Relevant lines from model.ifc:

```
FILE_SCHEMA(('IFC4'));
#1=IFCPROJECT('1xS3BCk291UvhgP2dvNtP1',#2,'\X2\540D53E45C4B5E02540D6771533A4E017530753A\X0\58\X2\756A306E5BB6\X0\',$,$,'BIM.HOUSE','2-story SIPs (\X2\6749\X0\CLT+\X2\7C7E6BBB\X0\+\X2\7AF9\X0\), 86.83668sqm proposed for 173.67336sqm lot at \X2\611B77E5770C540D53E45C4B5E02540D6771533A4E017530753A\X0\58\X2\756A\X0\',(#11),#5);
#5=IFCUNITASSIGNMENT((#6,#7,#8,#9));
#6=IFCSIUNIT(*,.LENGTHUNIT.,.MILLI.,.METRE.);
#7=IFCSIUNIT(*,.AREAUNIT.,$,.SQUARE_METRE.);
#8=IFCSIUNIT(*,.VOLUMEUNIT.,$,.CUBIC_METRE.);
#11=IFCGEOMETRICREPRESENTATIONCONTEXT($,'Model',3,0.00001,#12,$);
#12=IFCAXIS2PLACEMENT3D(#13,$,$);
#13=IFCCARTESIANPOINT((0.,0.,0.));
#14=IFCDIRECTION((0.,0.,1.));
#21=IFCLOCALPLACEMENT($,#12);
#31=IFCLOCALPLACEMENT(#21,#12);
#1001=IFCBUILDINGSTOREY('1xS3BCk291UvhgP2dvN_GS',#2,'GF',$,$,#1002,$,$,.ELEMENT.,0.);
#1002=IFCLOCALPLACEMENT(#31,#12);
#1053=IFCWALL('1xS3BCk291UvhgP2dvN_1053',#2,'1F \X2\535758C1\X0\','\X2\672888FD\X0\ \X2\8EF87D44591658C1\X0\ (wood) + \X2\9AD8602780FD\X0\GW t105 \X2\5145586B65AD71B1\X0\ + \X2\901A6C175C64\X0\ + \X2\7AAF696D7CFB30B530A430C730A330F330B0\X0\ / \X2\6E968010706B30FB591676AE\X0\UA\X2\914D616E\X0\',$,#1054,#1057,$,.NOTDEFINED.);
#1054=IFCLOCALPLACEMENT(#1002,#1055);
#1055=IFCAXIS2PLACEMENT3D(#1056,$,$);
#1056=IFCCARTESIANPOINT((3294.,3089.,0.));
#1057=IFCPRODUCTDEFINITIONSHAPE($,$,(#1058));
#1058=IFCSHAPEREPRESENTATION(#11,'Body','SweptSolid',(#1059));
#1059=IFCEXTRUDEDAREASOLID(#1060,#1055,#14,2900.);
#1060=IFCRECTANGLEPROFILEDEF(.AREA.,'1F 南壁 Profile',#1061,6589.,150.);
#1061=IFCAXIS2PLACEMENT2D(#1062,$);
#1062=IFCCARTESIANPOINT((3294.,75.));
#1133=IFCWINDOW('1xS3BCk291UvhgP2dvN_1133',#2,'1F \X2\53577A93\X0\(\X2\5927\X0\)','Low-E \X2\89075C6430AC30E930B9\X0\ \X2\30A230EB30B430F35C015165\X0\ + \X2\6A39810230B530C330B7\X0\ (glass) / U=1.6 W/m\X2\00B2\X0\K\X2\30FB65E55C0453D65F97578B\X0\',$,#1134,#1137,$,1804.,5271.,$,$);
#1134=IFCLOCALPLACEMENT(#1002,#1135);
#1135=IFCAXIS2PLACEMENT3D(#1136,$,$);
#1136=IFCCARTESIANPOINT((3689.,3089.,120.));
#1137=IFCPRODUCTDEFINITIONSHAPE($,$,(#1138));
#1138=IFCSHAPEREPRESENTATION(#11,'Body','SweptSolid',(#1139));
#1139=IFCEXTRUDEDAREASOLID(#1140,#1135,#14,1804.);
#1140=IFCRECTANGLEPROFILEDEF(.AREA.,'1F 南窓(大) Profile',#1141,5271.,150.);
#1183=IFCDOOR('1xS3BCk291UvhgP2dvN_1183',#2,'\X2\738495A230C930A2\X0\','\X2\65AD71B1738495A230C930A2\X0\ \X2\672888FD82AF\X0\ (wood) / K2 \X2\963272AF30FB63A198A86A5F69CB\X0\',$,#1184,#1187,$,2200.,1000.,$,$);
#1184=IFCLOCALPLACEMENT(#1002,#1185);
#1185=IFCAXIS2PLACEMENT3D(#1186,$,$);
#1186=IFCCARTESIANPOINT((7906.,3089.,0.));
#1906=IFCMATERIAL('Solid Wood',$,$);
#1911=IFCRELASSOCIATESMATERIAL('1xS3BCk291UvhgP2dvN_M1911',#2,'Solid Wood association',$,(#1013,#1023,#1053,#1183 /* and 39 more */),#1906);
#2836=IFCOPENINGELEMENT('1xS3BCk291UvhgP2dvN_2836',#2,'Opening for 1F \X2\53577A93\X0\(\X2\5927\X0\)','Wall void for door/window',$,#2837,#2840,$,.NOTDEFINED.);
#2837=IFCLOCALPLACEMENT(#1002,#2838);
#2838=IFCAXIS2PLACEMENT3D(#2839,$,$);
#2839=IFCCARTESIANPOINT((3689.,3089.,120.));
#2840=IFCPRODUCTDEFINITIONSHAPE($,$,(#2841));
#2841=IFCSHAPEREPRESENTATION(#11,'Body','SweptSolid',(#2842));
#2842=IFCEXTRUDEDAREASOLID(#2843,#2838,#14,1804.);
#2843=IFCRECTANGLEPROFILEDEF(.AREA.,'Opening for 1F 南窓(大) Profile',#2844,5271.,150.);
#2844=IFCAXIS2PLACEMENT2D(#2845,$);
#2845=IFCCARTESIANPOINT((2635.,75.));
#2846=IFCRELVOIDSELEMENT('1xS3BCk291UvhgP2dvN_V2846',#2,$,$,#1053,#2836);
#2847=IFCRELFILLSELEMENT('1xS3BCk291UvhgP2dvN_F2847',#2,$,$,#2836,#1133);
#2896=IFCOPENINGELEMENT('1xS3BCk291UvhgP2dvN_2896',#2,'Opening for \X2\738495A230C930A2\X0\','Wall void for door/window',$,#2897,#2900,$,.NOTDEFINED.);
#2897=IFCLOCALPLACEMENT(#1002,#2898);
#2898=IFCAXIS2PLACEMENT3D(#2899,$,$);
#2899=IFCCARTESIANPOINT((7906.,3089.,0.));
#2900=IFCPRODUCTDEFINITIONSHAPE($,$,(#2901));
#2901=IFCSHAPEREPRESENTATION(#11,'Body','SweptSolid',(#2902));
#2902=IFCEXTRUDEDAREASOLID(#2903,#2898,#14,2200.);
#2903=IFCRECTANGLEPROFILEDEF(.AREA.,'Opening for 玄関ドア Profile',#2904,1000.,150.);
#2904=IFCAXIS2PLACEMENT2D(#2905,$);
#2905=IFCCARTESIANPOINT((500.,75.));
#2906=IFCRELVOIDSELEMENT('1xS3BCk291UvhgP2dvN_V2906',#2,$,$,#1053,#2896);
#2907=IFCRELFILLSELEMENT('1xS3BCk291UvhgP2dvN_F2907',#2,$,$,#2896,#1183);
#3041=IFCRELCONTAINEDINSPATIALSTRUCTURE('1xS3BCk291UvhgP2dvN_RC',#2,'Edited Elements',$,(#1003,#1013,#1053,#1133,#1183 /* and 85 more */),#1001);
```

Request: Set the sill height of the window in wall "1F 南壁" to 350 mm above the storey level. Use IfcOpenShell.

```python
import numpy as np
import ifcopenshell
import ifcopenshell.api.geometry
import ifcopenshell.geom
import ifcopenshell.util.element
import ifcopenshell.util.placement
import ifcopenshell.util.shape
import ifcopenshell.util.unit

model = ifcopenshell.open("model.ifc")
unit_scale = ifcopenshell.util.unit.calculate_unit_scale(model)

window = model.by_guid("1xS3BCk291UvhgP2dvN_1133")
opening = window.FillsVoids[0].RelatingOpeningElement
storey = ifcopenshell.util.element.get_container(window, ifc_class="IfcBuildingStorey")
level = ifcopenshell.util.placement.get_local_placement(storey.ObjectPlacement)[2, 3]

# The opening's origin need not be at the sill, so measure its lowest point.
shape = ifcopenshell.geom.create_shape(ifcopenshell.geom.settings(), opening)
bottom = ifcopenshell.util.shape.get_shape_bottom_elevation(shape, shape.geometry) / unit_scale
dz = level + 0.35 / unit_scale - bottom

shift = np.array([0.0, 0.0, dz])
# The window is not placed relative to its opening, so move both.
for product in (opening, window):
    matrix = ifcopenshell.util.placement.get_local_placement(product.ObjectPlacement)
    matrix[:3, 3] += shift
    ifcopenshell.api.geometry.edit_object_placement(model, product=product, matrix=matrix, is_si=False)

print(f"moved by {dz * unit_scale:+.3f} m")

model.write("model_rev.ifc")
```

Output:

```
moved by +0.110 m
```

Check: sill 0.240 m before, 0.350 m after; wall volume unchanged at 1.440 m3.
